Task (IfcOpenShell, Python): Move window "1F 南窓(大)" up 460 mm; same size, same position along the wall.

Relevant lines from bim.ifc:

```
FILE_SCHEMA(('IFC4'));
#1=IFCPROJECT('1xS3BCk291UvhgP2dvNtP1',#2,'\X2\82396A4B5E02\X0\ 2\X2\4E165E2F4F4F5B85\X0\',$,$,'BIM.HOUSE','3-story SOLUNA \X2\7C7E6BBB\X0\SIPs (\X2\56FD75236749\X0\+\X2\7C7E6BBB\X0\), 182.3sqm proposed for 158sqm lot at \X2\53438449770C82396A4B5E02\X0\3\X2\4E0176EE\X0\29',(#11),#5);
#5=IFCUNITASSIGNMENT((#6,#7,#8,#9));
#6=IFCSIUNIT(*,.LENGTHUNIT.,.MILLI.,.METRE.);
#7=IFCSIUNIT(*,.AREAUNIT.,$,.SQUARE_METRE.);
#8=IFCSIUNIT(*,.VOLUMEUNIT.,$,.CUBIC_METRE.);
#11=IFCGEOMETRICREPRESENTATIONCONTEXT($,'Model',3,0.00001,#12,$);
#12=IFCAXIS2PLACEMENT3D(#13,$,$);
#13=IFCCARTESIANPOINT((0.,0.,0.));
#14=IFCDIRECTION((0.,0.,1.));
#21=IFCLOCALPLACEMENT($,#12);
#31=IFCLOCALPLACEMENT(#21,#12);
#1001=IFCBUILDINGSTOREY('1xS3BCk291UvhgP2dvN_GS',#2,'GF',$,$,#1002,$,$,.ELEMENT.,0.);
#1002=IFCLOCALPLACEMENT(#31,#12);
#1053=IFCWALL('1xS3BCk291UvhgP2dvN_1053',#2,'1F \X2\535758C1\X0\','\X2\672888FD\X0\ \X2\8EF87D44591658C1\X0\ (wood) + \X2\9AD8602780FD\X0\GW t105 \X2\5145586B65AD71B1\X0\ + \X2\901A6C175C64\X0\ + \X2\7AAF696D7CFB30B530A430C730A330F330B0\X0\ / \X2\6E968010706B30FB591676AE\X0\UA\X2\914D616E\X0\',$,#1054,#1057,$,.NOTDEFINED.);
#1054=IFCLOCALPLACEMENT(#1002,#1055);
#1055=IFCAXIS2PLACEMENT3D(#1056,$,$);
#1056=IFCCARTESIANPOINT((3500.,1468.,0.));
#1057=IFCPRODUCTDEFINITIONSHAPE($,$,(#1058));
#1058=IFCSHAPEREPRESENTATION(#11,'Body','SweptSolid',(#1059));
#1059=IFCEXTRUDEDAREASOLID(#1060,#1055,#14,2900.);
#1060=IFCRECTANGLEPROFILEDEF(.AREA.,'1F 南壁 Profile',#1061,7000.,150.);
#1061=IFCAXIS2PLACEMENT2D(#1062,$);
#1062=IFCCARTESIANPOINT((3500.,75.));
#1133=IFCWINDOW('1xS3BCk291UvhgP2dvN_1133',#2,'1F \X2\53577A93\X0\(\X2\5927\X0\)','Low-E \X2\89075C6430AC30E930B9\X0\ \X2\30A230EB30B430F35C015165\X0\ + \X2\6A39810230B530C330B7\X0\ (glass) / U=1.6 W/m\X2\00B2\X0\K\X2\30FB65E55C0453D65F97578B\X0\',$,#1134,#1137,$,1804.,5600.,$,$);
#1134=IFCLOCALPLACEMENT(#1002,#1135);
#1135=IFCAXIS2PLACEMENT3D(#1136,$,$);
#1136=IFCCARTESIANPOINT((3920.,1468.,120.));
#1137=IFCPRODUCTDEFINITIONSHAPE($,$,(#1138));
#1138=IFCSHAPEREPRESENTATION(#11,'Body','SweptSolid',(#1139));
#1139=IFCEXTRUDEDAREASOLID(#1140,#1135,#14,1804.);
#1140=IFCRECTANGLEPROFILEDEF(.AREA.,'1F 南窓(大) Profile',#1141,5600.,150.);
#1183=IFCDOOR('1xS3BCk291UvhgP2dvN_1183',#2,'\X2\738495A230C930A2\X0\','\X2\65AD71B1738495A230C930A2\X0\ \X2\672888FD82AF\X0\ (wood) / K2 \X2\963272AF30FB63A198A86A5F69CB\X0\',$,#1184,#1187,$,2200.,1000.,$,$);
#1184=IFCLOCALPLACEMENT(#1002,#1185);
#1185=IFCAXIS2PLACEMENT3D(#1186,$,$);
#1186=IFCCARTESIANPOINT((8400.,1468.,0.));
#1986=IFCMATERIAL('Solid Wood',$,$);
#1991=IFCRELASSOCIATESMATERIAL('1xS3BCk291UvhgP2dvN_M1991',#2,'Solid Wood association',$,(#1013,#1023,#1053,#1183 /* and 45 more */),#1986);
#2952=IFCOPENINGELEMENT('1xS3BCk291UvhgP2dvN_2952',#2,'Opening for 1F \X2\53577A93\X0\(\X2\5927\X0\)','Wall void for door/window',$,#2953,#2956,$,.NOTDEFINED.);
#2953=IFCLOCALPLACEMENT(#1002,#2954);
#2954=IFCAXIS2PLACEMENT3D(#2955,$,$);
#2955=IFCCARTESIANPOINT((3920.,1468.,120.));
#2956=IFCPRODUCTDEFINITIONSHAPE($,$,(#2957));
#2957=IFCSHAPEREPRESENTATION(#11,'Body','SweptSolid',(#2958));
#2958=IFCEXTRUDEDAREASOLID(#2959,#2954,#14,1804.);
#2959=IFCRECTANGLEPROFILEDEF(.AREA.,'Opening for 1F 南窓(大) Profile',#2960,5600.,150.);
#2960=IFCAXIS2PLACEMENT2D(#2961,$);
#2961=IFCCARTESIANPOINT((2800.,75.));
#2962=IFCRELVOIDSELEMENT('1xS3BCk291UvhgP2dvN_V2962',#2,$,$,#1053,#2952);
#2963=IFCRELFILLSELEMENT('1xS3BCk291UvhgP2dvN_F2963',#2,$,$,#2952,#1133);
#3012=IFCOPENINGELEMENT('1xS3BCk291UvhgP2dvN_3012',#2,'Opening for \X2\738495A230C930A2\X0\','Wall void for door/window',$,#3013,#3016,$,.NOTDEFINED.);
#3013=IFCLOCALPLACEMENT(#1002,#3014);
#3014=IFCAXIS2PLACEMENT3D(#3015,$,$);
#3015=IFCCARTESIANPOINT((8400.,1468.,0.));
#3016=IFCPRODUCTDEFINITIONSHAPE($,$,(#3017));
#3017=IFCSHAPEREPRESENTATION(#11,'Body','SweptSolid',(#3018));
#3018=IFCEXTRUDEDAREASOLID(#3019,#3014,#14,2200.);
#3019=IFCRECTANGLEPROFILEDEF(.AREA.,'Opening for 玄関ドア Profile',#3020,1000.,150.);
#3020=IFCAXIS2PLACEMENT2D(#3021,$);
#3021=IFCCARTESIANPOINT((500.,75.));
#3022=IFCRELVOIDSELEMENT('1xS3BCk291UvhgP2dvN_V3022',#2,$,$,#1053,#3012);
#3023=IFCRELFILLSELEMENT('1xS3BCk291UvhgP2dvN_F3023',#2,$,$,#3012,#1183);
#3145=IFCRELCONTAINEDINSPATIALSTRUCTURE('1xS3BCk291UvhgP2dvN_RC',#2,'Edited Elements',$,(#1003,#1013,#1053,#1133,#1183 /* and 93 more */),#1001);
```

```python
import numpy as np
import ifcopenshell
import ifcopenshell.api.geometry
import ifcopenshell.util.placement
import ifcopenshell.util.unit

model = ifcopenshell.open("bim.ifc")
unit_scale = ifcopenshell.util.unit.calculate_unit_scale(model)

window = model.by_guid("1xS3BCk291UvhgP2dvN_1133")
opening = window.FillsVoids[0].RelatingOpeningElement
dz = 0.46 / unit_scale

shift = np.array([0.0, 0.0, dz])
# The window is not placed relative to its opening, so move both.
for product in (opening, window):
    matrix = ifcopenshell.util.placement.get_local_placement(product.ObjectPlacement)
    matrix[:3, 3] += shift
    ifcopenshell.api.geometry.edit_object_placement(model, product=product, matrix=matrix, is_si=False)

print(f"moved by {dz * unit_scale:+.3f} m")

model.write("bim-out.ifc")
```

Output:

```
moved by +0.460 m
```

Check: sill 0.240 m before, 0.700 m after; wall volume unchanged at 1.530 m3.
